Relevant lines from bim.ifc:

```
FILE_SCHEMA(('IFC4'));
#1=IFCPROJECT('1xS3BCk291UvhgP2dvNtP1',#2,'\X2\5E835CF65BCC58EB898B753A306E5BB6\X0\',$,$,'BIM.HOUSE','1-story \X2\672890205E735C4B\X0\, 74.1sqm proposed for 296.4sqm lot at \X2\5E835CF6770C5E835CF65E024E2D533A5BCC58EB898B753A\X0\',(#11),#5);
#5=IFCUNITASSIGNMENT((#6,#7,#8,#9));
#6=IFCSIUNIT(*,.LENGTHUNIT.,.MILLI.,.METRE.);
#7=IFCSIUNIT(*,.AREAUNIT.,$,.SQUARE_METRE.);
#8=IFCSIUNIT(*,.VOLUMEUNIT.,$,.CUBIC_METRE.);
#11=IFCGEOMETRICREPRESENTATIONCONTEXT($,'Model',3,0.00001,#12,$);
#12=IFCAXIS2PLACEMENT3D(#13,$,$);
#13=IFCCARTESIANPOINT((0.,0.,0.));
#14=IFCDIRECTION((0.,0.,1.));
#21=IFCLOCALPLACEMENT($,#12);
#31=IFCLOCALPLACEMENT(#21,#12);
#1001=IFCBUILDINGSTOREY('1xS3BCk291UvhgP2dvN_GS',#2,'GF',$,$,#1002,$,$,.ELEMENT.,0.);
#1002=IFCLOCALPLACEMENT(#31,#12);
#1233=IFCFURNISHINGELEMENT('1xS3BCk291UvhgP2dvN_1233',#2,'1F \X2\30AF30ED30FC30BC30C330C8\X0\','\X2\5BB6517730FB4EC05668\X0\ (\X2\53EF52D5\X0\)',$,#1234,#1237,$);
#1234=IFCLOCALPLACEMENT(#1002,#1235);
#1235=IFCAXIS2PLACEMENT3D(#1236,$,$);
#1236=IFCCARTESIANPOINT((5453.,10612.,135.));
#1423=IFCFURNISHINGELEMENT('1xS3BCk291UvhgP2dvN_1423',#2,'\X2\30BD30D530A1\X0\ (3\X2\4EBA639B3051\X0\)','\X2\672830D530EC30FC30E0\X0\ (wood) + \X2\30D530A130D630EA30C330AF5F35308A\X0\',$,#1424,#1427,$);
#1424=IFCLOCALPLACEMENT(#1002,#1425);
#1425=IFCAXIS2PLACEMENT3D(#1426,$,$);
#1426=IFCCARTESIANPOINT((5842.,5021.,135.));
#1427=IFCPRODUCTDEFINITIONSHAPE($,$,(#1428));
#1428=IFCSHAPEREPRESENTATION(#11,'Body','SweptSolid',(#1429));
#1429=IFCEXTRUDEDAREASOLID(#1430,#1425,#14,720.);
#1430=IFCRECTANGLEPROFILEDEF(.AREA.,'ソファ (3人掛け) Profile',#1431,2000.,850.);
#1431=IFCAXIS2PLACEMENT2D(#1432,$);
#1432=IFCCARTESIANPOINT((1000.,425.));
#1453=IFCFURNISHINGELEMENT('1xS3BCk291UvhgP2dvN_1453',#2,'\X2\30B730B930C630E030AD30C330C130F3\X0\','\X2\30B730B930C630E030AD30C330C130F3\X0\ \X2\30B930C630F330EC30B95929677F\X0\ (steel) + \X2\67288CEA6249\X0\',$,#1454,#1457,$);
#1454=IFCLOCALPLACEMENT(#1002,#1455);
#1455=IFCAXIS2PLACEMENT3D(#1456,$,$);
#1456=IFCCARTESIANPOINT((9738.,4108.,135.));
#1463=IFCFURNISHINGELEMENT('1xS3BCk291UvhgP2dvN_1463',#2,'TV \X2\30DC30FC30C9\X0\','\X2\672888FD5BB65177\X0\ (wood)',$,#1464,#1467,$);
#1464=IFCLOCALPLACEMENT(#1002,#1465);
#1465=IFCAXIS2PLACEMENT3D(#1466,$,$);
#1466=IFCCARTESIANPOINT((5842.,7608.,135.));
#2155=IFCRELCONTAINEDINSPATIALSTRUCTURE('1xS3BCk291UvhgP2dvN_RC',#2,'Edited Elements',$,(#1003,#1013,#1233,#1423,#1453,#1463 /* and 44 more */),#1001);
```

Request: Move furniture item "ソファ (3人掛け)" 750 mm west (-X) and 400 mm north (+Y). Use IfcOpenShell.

```python
import ifcopenshell
import ifcopenshell.api.geometry
import ifcopenshell.util.placement
import ifcopenshell.util.unit

model = ifcopenshell.open("bim.ifc")
unit_scale = ifcopenshell.util.unit.calculate_unit_scale(model)

item = model.by_id(1423)
matrix = ifcopenshell.util.placement.get_local_placement(item.ObjectPlacement)
matrix[0, 3] -= 0.75 / unit_scale
matrix[1, 3] += 0.4 / unit_scale
ifcopenshell.api.geometry.edit_object_placement(model, product=item, matrix=matrix, is_si=False)

print(ifcopenshell.util.placement.get_local_placement(item.ObjectPlacement).round(3) + 0.0)

model.write("bim_edited.ifc")
```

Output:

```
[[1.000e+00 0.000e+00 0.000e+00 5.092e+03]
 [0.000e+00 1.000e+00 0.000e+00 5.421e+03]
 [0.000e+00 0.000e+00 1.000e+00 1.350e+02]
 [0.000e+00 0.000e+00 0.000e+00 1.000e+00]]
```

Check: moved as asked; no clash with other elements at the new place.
